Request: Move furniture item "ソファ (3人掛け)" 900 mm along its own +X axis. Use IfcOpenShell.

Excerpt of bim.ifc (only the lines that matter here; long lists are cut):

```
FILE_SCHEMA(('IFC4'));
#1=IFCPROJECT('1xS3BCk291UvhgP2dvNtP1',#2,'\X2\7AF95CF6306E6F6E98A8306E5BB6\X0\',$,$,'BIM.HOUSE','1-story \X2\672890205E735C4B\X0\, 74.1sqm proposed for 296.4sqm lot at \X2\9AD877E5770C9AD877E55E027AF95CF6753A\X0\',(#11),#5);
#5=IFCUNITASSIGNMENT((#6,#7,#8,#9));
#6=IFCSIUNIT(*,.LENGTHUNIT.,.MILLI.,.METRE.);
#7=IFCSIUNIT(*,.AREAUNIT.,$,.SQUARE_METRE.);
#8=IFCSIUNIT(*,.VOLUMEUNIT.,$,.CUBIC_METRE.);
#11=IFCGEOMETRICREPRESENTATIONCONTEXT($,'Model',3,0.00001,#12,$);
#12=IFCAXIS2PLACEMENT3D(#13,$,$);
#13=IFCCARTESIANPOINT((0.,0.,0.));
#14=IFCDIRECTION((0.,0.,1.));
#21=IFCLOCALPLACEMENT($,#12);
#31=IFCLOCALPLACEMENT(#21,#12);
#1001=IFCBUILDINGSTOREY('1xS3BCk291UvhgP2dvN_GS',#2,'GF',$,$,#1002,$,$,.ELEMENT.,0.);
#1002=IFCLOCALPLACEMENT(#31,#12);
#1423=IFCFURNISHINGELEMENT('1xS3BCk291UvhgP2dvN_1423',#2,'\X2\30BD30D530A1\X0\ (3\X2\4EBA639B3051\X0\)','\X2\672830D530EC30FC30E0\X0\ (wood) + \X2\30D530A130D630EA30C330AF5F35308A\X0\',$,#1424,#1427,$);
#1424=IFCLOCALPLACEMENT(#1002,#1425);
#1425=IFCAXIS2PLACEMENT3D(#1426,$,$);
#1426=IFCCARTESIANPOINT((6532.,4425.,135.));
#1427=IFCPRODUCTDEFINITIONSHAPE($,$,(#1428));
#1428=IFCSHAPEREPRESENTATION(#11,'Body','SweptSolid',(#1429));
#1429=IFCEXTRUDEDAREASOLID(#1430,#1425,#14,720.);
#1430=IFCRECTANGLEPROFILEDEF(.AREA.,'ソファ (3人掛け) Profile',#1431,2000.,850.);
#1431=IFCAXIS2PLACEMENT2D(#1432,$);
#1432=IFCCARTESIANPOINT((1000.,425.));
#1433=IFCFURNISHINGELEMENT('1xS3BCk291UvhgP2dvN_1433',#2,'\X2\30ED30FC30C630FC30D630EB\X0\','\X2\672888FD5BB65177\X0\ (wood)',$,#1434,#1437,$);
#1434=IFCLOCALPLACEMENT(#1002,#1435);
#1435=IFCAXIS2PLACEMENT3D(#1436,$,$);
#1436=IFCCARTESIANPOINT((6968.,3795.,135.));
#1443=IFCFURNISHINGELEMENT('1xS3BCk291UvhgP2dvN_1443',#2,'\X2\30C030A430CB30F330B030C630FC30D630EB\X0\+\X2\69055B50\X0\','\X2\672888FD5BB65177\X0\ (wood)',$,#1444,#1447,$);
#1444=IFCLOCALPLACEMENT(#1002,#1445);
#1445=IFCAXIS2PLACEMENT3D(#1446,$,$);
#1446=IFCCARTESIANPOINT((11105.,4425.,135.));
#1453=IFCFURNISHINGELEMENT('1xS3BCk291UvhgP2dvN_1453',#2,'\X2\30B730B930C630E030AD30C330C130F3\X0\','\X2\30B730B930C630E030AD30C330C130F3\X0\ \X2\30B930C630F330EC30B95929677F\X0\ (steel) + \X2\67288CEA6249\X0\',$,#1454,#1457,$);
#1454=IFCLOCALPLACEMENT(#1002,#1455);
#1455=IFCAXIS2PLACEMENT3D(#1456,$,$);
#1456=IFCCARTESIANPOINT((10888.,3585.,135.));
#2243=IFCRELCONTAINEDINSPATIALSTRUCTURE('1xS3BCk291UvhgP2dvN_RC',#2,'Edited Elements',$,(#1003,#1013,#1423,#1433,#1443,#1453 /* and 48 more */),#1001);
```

```python
import ifcopenshell
import ifcopenshell.api.geometry
import ifcopenshell.util.placement
import ifcopenshell.util.unit

model = ifcopenshell.open("bim.ifc")
unit_scale = ifcopenshell.util.unit.calculate_unit_scale(model)

item = model.by_guid("1xS3BCk291UvhgP2dvN_1423")
matrix = ifcopenshell.util.placement.get_local_placement(item.ObjectPlacement)
matrix[:3, 3] += matrix[:3, 0] * 0.9 / unit_scale
ifcopenshell.api.geometry.edit_object_placement(model, product=item, matrix=matrix, is_si=False)

print(ifcopenshell.util.placement.get_local_placement(item.ObjectPlacement).round(3) + 0.0)

model.write("bim_edited.ifc")
```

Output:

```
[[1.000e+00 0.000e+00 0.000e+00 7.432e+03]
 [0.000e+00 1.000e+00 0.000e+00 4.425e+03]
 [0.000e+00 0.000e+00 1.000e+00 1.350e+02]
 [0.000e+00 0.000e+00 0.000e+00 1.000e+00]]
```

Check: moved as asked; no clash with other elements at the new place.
